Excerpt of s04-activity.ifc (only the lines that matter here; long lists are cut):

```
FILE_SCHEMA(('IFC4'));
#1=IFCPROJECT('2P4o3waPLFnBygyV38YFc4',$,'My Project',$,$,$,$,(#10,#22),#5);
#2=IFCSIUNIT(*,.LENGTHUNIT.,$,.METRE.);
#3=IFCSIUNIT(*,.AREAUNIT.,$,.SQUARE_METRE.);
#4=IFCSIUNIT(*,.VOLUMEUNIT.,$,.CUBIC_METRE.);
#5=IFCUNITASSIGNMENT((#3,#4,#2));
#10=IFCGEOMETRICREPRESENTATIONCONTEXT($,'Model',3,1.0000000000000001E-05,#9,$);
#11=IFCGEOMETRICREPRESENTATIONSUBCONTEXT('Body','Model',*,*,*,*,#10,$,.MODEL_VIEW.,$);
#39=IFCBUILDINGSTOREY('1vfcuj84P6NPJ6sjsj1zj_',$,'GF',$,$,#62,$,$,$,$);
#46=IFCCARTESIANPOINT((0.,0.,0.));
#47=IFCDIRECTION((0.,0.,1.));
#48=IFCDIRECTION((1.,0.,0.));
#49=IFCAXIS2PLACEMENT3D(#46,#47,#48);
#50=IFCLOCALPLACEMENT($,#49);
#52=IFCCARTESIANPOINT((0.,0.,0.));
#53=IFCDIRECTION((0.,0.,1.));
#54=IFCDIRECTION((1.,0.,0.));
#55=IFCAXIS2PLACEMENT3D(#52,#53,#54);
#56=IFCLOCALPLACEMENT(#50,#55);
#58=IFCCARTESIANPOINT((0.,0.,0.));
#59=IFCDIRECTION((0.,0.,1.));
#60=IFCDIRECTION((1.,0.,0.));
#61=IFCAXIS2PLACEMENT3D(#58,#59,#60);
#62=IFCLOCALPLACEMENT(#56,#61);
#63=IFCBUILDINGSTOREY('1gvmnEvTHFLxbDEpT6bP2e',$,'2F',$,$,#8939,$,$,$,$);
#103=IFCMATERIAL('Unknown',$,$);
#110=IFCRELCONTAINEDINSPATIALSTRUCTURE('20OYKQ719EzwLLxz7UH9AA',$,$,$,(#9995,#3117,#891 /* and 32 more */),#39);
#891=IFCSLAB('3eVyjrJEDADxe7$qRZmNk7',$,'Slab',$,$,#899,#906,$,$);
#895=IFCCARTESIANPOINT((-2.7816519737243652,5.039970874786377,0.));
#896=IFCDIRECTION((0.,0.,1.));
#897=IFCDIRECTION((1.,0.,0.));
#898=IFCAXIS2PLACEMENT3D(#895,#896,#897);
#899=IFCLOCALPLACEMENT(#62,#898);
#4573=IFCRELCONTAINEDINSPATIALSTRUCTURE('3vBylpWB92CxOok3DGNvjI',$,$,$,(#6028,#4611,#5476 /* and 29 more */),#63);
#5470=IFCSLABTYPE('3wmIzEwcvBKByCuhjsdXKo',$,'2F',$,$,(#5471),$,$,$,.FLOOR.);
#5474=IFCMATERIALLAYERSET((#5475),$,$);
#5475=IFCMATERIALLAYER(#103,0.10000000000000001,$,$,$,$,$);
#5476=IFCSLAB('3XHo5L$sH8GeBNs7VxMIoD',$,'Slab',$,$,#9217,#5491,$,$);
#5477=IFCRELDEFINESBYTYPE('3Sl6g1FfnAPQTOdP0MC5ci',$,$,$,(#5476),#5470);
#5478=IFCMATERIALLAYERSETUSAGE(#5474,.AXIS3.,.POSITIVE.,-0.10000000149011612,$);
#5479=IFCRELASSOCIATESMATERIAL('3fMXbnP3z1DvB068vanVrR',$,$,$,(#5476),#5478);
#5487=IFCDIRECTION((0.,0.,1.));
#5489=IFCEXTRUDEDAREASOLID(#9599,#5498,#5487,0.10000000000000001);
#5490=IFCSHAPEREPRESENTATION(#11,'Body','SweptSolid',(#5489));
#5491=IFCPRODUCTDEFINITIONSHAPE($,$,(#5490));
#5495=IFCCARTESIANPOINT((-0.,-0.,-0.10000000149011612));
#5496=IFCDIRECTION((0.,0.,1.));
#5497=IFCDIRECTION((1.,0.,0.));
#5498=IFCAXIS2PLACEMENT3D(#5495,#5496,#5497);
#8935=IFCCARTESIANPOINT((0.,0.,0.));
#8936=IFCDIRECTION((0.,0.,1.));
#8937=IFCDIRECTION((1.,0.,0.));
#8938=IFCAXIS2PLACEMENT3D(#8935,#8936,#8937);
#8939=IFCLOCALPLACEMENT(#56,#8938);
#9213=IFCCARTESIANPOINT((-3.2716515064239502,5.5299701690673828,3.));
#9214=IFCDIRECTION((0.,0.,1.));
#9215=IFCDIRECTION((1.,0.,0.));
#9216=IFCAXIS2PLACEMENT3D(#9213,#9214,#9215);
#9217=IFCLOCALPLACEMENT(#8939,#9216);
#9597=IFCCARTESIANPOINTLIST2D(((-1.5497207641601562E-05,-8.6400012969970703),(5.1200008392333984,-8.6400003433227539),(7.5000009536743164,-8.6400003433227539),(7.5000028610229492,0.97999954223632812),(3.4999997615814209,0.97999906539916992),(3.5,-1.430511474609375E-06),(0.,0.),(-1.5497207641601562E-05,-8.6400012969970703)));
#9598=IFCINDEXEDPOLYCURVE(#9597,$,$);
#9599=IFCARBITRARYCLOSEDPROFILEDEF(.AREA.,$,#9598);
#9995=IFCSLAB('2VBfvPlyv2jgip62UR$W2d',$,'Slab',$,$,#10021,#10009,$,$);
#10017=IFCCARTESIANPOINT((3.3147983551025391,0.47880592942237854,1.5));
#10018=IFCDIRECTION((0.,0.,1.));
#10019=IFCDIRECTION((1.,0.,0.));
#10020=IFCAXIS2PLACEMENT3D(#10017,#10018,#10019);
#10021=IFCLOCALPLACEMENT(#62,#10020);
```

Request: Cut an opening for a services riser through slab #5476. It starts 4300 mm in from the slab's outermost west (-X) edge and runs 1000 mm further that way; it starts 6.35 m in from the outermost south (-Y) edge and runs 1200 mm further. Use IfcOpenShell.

```python
import numpy as np
import ifcopenshell
import ifcopenshell.api.feature
import ifcopenshell.api.geometry
import ifcopenshell.api.root
import ifcopenshell.geom
import ifcopenshell.util.placement
import ifcopenshell.util.representation
import ifcopenshell.util.shape
import ifcopenshell.util.unit

model = ifcopenshell.open("s04-activity.ifc")
unit_scale = ifcopenshell.util.unit.calculate_unit_scale(model)
settings = ifcopenshell.geom.settings()


def volume(element):
    """Net volume in cubic metres, openings subtracted."""
    shape = ifcopenshell.geom.create_shape(settings, element)
    return ifcopenshell.util.shape.get_volume(shape.geometry)


slab = model.by_id(5476)
before = volume(slab)

# Extent in the slab's own axes, in metres. The edges named are its -X and -Y sides.
slab_shape = ifcopenshell.geom.create_shape(settings, slab)
vertices = ifcopenshell.util.shape.get_vertices(slab_shape.geometry)
x_min, y_min, bottom = vertices.min(axis=0)
top = vertices[:, 2].max()

opening = ifcopenshell.api.root.create_entity(model, ifc_class="IfcOpeningElement", name="Services riser opening", predefined_type="OPENING")
context = ifcopenshell.util.representation.get_context(model, "Model", "Body", "MODEL_VIEW")
width, depth = 1, 1.2
outline = [(0.0, 0.0), (width, 0.0), (width, depth), (0.0, depth), (0.0, 0.0)]
# Overshoot both faces by 50 mm so the cut is clean.
shape = ifcopenshell.api.geometry.add_slab_representation(
    model, context=context, depth=top - bottom + 0.1, polyline=outline
)
ifcopenshell.api.geometry.assign_representation(model, product=opening, representation=shape)

matrix = ifcopenshell.util.placement.get_local_placement(slab.ObjectPlacement)
matrix[:, 3] = matrix @ np.append(np.array([x_min + 4.3, y_min + 6.35, bottom - 0.05]) / unit_scale, 1.0)
ifcopenshell.api.geometry.edit_object_placement(model, product=opening, matrix=matrix, is_si=False)
ifcopenshell.api.feature.add_feature(model, feature=opening, element=slab)

after = volume(slab)

print(f"slab volume {before:.3f} -> {after:.3f} m3")

model.write("s04-activity-out.ifc")
```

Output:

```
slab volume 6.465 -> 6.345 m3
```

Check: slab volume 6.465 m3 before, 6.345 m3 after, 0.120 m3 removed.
